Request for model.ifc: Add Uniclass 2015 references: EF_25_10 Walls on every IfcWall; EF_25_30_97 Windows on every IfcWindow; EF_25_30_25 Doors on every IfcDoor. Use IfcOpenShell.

First a look at what the model holds.

```python
import ifcopenshell

model = ifcopenshell.open("model.ifc")
print(model.schema)
print("classifications:", [c.Name for c in model.by_type("IfcClassification")])
for ifc_class in ("IfcDoor", "IfcRoof", "IfcStair", "IfcWall", "IfcWindow"):
    print(ifc_class, len(model.by_type(ifc_class)))
```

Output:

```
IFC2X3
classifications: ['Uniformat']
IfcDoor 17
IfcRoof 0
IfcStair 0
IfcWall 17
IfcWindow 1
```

```python
import ifcopenshell
import ifcopenshell.api.classification

model = ifcopenshell.open("model.ifc")

# IFC2X3 requires Source and Edition and has no link from the project to the system.
system = model.create_entity("IfcClassification", Source="NBS", Edition="2015", Name="Uniclass 2015")

codes = {
    "IfcWall": ("EF_25_10", "Walls"),
    "IfcWindow": ("EF_25_30_97", "Windows"),
    "IfcDoor": ("EF_25_30_25", "Doors"),
}
for ifc_class, (code, name) in codes.items():
    products = model.by_type(ifc_class)
    ifcopenshell.api.classification.add_reference(
        model, products=products, classification=system, identification=code, name=name
    )
    print(code, len(products))

model.write("model_edited.ifc")
```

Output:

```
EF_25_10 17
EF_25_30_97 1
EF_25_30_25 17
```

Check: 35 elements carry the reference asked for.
